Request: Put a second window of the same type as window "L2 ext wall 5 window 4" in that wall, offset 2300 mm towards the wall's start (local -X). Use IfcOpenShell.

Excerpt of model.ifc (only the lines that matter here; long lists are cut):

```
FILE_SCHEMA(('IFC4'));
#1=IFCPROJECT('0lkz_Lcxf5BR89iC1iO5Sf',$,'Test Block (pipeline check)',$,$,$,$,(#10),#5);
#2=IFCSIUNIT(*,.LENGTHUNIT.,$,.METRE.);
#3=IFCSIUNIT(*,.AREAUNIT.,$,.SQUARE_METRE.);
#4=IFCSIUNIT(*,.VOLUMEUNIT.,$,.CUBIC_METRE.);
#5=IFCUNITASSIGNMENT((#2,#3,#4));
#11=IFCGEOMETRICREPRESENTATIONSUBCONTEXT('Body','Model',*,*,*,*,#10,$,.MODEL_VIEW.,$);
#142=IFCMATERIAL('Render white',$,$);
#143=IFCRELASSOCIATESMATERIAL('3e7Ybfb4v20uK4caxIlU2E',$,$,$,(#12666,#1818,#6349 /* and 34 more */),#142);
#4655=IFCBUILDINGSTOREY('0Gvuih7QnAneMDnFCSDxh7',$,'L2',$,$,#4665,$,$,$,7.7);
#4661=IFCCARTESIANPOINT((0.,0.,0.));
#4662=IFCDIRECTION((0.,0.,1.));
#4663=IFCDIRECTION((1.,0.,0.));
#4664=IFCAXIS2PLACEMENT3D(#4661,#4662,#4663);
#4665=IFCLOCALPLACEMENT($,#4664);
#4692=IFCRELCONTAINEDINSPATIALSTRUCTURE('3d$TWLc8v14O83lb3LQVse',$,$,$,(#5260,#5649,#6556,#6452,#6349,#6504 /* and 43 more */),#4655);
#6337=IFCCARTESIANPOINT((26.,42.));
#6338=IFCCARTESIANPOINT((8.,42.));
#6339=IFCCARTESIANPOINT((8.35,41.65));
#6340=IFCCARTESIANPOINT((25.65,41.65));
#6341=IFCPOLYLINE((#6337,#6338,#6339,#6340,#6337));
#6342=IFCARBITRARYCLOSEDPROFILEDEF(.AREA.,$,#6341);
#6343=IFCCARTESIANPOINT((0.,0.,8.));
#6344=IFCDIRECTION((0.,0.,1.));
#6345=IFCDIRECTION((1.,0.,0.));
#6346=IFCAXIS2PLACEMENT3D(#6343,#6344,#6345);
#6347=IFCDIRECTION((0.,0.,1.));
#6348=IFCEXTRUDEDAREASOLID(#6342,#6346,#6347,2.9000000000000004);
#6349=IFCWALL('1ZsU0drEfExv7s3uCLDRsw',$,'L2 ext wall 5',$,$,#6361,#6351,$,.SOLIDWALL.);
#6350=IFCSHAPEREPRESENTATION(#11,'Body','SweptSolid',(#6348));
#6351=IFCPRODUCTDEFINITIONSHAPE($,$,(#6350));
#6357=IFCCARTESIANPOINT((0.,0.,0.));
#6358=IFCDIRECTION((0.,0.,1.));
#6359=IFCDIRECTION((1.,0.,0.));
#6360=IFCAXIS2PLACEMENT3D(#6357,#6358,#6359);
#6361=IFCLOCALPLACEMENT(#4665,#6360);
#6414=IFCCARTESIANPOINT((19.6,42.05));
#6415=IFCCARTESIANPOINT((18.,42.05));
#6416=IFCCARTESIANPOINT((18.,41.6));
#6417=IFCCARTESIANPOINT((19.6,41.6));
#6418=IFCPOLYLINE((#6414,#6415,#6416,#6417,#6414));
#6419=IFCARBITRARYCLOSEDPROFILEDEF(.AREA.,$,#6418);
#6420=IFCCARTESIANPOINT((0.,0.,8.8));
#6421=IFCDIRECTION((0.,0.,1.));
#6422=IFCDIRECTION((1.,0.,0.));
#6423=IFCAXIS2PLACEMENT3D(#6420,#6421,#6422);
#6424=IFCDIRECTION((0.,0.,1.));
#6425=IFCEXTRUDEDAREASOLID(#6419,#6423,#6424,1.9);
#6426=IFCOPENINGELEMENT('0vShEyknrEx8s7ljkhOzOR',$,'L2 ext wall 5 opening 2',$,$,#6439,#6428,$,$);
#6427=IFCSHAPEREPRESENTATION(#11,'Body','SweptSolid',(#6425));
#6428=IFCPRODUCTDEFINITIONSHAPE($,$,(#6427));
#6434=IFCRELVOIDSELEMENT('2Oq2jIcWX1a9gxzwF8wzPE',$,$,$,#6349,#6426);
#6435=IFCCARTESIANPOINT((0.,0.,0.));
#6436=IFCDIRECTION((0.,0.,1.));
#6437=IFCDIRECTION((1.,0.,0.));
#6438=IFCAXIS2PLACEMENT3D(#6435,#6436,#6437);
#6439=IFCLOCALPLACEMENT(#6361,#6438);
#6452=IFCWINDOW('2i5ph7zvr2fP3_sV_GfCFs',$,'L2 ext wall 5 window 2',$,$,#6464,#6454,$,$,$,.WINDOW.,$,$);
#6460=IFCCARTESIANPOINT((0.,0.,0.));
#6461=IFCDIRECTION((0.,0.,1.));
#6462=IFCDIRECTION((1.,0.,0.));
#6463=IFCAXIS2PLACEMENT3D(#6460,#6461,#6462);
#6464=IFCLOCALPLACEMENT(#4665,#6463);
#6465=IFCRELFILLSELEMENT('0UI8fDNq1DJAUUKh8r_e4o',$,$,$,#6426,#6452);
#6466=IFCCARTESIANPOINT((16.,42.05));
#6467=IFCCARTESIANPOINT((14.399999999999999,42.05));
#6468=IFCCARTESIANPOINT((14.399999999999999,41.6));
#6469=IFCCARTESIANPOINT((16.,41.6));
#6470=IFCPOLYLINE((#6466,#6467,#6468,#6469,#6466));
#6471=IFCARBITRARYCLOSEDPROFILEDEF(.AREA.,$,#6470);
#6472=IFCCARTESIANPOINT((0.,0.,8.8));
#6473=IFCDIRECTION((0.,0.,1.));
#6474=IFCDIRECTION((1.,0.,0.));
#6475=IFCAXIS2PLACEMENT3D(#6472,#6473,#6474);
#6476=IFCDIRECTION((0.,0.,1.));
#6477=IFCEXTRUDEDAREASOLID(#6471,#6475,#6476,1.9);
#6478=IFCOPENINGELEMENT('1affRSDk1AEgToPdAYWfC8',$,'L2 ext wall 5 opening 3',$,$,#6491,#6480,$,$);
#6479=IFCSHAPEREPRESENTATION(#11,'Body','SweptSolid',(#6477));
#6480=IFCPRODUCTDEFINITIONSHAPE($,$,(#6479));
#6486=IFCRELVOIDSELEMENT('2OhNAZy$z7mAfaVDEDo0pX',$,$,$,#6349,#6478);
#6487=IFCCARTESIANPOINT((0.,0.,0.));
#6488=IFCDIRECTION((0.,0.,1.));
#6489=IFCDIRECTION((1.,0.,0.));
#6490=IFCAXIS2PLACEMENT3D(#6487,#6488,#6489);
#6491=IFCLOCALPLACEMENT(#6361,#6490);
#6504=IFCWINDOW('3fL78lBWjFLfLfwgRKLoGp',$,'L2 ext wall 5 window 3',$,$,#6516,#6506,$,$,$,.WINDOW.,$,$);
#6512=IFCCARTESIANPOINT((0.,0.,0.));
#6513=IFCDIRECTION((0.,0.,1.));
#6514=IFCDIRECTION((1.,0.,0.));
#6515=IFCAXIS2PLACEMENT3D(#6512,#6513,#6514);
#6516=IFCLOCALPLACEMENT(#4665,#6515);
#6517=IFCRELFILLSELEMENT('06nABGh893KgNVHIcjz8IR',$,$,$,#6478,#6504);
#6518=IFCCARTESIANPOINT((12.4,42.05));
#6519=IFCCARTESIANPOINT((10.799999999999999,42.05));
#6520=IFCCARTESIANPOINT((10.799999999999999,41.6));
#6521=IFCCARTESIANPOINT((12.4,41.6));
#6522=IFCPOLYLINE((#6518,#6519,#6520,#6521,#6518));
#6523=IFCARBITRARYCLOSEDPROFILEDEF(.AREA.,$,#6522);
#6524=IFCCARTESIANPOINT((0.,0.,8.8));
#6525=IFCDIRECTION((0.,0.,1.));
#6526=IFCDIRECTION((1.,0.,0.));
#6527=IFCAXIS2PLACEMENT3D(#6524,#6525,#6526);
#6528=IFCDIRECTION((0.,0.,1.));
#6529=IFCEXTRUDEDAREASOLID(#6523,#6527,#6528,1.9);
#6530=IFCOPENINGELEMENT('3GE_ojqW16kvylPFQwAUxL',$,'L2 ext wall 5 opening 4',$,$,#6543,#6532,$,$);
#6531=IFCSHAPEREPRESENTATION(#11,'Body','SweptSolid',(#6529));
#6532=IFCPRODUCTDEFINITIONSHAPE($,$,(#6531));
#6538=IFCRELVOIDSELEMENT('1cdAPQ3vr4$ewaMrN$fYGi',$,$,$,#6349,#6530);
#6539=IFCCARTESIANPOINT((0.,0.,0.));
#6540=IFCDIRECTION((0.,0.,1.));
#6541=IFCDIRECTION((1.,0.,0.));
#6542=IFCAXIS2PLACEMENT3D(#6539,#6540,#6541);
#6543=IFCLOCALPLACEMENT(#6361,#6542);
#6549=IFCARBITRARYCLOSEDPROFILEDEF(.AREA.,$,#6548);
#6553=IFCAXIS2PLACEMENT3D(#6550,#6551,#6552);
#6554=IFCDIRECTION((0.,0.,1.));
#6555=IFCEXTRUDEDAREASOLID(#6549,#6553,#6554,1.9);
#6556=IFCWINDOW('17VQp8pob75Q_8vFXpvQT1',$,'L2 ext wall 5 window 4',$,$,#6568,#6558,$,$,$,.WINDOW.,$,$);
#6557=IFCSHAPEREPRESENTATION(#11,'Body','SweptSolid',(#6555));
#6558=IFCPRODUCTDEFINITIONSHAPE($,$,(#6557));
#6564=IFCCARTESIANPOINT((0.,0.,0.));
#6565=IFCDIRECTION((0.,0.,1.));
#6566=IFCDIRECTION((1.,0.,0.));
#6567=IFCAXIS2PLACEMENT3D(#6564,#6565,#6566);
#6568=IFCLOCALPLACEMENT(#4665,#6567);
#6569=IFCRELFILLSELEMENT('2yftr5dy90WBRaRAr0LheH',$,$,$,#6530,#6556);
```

```python
import ifcopenshell
import ifcopenshell.api.feature
import ifcopenshell.api.geometry
import ifcopenshell.api.root
import ifcopenshell.geom
import ifcopenshell.util.element
import ifcopenshell.util.placement
import ifcopenshell.util.shape

model = ifcopenshell.open("model.ifc")
settings = ifcopenshell.geom.settings()


def volume(element):
    """Net volume in cubic metres, openings subtracted."""
    shape = ifcopenshell.geom.create_shape(settings, element)
    return ifcopenshell.util.shape.get_volume(shape.geometry)


window = model.by_guid("17VQp8pob75Q_8vFXpvQT1")
opening = window.FillsVoids[0].RelatingOpeningElement
wall = opening.VoidsElements[0].RelatingBuildingElement
before = volume(wall)
shift = ifcopenshell.util.placement.get_local_placement(wall.ObjectPlacement)[:3, 0] * -2.3

# copy_class copies the void relationship, type, container and properties, but no geometry.
new_opening = ifcopenshell.api.root.copy_class(model, product=opening)
new_opening.Representation = ifcopenshell.util.element.copy_deep(
    model, opening.Representation, exclude=["IfcGeometricRepresentationContext", "IfcRepresentationMap"]
)
new_window = ifcopenshell.api.root.copy_class(model, product=window)
new_window.Representation = ifcopenshell.util.element.copy_deep(
    model, window.Representation, exclude=["IfcGeometricRepresentationContext", "IfcRepresentationMap"]
)
ifcopenshell.api.feature.add_filling(model, opening=new_opening, element=new_window)

for old, new in ((opening, new_opening), (window, new_window)):
    matrix = ifcopenshell.util.placement.get_local_placement(old.ObjectPlacement)
    matrix[:3, 3] += shift
    ifcopenshell.api.geometry.edit_object_placement(model, product=new, matrix=matrix, is_si=False)

after = volume(wall)

print(f"wall volume {before:.3f} -> {after:.3f} m3")

model.write("model-out.ifc")
```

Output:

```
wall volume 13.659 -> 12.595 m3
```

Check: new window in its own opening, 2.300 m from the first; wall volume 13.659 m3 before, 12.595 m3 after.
